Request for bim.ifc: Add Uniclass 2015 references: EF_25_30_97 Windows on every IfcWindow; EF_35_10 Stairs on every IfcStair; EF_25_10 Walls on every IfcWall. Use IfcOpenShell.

First a look at what the model holds.

```python
import ifcopenshell

model = ifcopenshell.open("bim.ifc")
print(model.schema)
print("classifications:", [c.Name for c in model.by_type("IfcClassification")])
for ifc_class in ("IfcDoor", "IfcRoof", "IfcStair", "IfcWall", "IfcWindow"):
    print(ifc_class, len(model.by_type(ifc_class)))
```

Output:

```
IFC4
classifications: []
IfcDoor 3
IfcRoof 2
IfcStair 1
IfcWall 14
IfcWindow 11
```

```python
import ifcopenshell
import ifcopenshell.api.classification

model = ifcopenshell.open("bim.ifc")

system = ifcopenshell.api.classification.add_classification(model, classification="Uniclass 2015")

codes = {
    "IfcWindow": ("EF_25_30_97", "Windows"),
    "IfcStair": ("EF_35_10", "Stairs"),
    "IfcWall": ("EF_25_10", "Walls"),
}
for ifc_class, (code, name) in codes.items():
    products = model.by_type(ifc_class)
    ifcopenshell.api.classification.add_reference(
        model, products=products, classification=system, identification=code, name=name
    )
    print(code, len(products))

model.write("bim_updated.ifc")
```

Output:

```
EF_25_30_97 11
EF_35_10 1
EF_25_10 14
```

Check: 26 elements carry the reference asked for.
